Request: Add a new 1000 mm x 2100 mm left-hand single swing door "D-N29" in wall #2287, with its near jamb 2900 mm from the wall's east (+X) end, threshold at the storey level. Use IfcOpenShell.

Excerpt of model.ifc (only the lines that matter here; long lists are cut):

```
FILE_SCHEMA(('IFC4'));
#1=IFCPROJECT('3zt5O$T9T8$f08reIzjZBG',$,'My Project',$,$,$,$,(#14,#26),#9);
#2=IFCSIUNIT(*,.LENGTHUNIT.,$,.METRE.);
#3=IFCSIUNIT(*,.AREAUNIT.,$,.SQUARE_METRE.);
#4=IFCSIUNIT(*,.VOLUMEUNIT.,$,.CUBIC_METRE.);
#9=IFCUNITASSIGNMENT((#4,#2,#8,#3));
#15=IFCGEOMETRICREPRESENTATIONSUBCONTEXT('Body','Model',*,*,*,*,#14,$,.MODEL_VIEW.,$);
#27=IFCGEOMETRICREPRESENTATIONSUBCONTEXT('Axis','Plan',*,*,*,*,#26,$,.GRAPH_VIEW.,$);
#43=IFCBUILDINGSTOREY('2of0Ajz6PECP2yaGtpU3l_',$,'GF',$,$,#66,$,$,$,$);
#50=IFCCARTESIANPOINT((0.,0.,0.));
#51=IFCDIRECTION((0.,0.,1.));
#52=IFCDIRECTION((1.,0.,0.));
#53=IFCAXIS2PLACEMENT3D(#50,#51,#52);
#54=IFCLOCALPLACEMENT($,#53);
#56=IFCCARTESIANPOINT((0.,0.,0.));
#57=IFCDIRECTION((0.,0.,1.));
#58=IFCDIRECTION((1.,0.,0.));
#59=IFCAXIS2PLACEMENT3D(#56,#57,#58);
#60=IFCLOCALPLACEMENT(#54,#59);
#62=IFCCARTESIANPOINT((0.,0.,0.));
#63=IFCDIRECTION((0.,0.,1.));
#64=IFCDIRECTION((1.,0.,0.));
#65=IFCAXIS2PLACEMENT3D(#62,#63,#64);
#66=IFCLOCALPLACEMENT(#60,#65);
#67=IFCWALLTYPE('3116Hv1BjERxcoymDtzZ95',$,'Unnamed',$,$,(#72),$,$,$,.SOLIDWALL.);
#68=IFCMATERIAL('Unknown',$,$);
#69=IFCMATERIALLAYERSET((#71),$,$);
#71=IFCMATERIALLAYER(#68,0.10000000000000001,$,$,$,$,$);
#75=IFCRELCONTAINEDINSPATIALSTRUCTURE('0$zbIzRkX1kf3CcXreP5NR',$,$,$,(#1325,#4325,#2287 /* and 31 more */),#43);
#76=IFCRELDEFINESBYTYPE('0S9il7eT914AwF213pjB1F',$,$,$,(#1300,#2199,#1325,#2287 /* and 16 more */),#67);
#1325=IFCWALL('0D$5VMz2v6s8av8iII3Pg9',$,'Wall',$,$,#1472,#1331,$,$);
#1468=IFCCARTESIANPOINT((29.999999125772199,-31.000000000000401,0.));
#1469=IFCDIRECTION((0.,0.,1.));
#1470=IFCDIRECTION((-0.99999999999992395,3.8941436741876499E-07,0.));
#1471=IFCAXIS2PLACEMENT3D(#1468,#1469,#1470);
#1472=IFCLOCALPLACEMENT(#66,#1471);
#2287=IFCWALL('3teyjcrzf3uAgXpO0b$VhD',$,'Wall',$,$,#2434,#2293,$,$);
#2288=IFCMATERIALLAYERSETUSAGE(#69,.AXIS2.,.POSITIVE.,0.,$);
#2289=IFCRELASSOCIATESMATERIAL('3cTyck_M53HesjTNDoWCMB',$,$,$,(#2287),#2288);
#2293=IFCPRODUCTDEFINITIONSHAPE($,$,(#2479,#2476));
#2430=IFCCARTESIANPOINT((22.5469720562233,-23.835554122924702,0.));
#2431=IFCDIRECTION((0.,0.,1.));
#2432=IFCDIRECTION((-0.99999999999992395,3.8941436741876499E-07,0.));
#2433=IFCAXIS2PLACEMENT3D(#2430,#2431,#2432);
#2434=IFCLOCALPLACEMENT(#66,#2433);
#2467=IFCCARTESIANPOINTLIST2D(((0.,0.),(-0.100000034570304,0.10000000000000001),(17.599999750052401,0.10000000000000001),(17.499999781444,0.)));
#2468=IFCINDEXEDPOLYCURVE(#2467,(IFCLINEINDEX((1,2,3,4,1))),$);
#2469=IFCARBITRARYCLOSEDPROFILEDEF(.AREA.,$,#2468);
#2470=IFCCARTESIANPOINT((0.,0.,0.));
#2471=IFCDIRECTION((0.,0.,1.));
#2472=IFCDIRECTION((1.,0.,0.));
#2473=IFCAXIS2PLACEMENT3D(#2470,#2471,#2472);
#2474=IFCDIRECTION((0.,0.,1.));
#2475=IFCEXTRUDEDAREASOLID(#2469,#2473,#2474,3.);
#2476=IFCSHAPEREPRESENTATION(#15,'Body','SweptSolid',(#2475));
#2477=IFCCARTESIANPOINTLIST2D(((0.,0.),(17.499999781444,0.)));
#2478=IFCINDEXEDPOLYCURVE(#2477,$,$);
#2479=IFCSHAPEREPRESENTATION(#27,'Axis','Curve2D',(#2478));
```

```python
import numpy as np
import ifcopenshell
import ifcopenshell.api.feature
import ifcopenshell.api.geometry
import ifcopenshell.api.root
import ifcopenshell.api.spatial
import ifcopenshell.geom
import ifcopenshell.util.element
import ifcopenshell.util.placement
import ifcopenshell.util.representation
import ifcopenshell.util.shape
import ifcopenshell.util.unit

model = ifcopenshell.open("model.ifc")
unit_scale = ifcopenshell.util.unit.calculate_unit_scale(model)
settings = ifcopenshell.geom.settings()


def volume(element):
    """Net volume in cubic metres, openings subtracted."""
    shape = ifcopenshell.geom.create_shape(settings, element)
    return ifcopenshell.util.shape.get_volume(shape.geometry)


wall = model.by_id(2287)
storey = ifcopenshell.util.element.get_container(wall, ifc_class="IfcBuildingStorey")
context = ifcopenshell.util.representation.get_context(model, "Model", "Body", "MODEL_VIEW")
before = volume(wall)

width, height, from_end, sill = 1, 2.1, 2.9, 0.0  # metres

# The wall runs along its own X axis, and the end named is its -X end.
wall_shape = ifcopenshell.geom.create_shape(settings, wall)
x, y, z = ifcopenshell.util.shape.get_vertices(wall_shape.geometry).T
start = x.min() + from_end
face, thickness = float(y.min()), float(y.max() - y.min())
wall_matrix = ifcopenshell.util.placement.get_local_placement(wall.ObjectPlacement)
level = ifcopenshell.util.placement.get_local_placement(storey.ObjectPlacement)[2, 3]


def in_wall(x, y):
    """Placement at x, y metres in the wall's axes, at sill height."""
    matrix = wall_matrix.copy()
    matrix[:, 3] = wall_matrix @ np.array([x / unit_scale, y / unit_scale, 0.0, 1.0])
    matrix[2, 3] = level + sill / unit_scale
    return matrix


# Opening: a box that overshoots both wall faces by 50 mm.
opening = ifcopenshell.api.root.create_entity(model, ifc_class="IfcOpeningElement", predefined_type="OPENING")
box = ifcopenshell.api.geometry.add_wall_representation(
    model, context=context, length=width, height=height, thickness=thickness + 0.1
)
ifcopenshell.api.geometry.assign_representation(model, product=opening, representation=box)
ifcopenshell.api.geometry.edit_object_placement(model, product=opening, matrix=in_wall(start, face - 0.05), is_si=False)
ifcopenshell.api.feature.add_feature(model, feature=opening, element=wall)

door = ifcopenshell.api.root.create_entity(model, ifc_class="IfcDoor", name="D-N29", predefined_type="DOOR")
door.OverallWidth, door.OverallHeight = width / unit_scale, height / unit_scale
door.OperationType = "SINGLE_SWING_LEFT"
body = ifcopenshell.api.geometry.add_door_representation(
    model,
    context=context,
    overall_width=door.OverallWidth,
    overall_height=door.OverallHeight,
    operation_type="SINGLE_SWING_LEFT",
    lining_properties={"LiningDepth": thickness / unit_scale, "ThresholdDepth": thickness / unit_scale},
)
ifcopenshell.api.geometry.assign_representation(model, product=door, representation=body)
ifcopenshell.api.spatial.assign_container(model, products=[door], relating_structure=storey)
ifcopenshell.api.feature.add_filling(model, opening=opening, element=door)

# The lining spans the wall, so the door starts at the wall face.
ifcopenshell.api.geometry.edit_object_placement(model, product=door, matrix=in_wall(start, face), is_si=False)

after = volume(wall)

print(f"wall volume {before:.3f} -> {after:.3f} m3")

model.write("model_updated.ifc")
```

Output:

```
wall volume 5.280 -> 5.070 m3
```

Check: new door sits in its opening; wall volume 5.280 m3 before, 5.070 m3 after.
